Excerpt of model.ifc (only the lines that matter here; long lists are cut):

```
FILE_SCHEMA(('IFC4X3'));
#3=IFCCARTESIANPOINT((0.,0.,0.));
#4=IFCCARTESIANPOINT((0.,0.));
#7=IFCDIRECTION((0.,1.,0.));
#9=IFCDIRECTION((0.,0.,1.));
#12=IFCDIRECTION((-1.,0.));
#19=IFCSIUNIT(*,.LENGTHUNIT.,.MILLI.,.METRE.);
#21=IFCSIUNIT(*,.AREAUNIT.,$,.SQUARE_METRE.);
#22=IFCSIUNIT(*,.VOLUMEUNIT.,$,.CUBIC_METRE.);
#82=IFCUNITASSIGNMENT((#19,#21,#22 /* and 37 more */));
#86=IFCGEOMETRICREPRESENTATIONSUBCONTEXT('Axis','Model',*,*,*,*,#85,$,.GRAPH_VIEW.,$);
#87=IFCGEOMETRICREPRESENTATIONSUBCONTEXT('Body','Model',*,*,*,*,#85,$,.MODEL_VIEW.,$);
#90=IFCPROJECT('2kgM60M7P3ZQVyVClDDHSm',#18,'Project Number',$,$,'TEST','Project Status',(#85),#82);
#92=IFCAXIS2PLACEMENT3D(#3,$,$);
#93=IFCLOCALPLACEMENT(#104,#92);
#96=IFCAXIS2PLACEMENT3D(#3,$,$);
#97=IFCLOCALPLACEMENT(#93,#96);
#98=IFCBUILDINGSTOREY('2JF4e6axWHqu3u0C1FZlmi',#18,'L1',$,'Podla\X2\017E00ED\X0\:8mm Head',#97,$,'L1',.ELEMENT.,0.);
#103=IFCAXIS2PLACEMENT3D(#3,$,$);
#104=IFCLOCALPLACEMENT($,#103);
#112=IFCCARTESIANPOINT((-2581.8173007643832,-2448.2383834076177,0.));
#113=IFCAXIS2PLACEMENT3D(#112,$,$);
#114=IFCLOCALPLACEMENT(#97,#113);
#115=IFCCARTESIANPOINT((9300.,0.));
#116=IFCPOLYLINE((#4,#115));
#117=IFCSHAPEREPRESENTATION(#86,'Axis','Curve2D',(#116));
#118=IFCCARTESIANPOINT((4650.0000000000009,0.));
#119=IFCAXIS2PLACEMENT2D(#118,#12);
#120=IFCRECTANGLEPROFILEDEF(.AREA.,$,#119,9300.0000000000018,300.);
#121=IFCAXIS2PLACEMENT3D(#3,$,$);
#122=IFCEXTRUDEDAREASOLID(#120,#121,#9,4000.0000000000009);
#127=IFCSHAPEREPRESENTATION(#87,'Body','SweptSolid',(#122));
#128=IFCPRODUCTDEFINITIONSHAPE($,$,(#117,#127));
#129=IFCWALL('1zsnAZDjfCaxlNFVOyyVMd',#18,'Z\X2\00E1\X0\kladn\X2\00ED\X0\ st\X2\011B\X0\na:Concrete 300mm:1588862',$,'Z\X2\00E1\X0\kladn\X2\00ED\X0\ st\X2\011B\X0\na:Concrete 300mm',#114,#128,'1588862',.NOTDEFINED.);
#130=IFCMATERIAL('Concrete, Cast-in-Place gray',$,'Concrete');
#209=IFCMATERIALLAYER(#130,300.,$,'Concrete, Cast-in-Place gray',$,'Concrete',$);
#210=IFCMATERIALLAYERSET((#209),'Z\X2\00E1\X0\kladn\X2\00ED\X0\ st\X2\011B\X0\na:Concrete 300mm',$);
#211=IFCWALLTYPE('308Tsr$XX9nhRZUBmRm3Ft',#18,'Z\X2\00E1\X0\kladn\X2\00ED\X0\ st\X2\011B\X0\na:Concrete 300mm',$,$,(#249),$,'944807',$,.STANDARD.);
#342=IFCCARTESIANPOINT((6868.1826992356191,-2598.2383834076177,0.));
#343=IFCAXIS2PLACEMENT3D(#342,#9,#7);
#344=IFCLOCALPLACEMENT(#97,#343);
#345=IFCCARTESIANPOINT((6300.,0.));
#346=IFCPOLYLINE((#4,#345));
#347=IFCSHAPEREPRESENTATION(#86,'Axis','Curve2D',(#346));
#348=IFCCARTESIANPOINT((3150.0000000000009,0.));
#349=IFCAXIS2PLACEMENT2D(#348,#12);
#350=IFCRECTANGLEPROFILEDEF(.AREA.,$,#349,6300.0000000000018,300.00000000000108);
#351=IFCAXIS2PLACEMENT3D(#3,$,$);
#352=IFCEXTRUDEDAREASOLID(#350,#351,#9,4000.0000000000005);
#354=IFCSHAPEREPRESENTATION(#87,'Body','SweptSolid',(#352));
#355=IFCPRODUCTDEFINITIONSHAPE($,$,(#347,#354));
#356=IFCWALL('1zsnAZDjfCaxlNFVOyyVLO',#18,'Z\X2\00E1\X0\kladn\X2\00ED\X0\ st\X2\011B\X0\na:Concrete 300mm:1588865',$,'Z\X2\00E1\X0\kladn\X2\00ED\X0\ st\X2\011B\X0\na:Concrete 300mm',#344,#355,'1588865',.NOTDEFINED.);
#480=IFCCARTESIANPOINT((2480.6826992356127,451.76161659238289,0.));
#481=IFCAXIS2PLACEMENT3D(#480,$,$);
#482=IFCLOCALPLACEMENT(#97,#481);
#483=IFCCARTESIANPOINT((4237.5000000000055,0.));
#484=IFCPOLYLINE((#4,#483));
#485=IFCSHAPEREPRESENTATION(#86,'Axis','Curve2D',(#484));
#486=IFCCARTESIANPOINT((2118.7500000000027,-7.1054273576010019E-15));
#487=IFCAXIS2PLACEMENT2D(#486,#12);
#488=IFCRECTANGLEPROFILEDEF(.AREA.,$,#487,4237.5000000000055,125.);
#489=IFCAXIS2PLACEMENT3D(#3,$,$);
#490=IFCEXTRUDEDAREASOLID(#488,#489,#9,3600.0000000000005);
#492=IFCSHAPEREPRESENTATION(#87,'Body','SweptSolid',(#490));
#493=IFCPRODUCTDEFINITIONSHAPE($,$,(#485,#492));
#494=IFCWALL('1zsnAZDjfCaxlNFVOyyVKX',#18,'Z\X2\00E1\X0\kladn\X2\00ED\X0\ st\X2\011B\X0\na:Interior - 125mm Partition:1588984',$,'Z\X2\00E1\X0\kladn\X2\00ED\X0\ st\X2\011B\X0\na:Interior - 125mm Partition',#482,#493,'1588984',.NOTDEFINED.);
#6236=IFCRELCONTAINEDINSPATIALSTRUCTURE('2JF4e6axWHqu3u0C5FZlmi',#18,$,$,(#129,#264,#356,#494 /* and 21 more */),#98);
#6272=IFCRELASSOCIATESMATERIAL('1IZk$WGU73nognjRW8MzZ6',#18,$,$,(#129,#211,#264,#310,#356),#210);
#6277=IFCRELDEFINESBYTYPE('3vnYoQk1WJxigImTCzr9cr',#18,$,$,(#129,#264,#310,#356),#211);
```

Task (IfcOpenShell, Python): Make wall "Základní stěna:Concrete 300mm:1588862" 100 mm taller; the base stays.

```python
import ifcopenshell
import ifcopenshell.geom
import ifcopenshell.util.representation
import ifcopenshell.util.shape
import ifcopenshell.util.unit

model = ifcopenshell.open("model.ifc")
unit_scale = ifcopenshell.util.unit.calculate_unit_scale(model)
settings = ifcopenshell.geom.settings()


def volume(element):
    """Net volume in cubic metres, openings subtracted."""
    shape = ifcopenshell.geom.create_shape(settings, element)
    return ifcopenshell.util.shape.get_volume(shape.geometry)


wall = model.by_guid("1zsnAZDjfCaxlNFVOyyVMd")
before = volume(wall)

body = ifcopenshell.util.representation.get_representation(wall, "Model", "Body")
solid = body.Items[0]
old_height = solid.Depth
solid.Depth += 0.1 / unit_scale
after = volume(wall)

print(f"height {old_height:g} -> {solid.Depth:g}, volume {before:.3f} -> {after:.3f} m3")

model.write("model_updated.ifc")
```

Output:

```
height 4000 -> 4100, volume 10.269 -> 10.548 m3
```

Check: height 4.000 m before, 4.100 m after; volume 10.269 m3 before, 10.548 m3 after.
